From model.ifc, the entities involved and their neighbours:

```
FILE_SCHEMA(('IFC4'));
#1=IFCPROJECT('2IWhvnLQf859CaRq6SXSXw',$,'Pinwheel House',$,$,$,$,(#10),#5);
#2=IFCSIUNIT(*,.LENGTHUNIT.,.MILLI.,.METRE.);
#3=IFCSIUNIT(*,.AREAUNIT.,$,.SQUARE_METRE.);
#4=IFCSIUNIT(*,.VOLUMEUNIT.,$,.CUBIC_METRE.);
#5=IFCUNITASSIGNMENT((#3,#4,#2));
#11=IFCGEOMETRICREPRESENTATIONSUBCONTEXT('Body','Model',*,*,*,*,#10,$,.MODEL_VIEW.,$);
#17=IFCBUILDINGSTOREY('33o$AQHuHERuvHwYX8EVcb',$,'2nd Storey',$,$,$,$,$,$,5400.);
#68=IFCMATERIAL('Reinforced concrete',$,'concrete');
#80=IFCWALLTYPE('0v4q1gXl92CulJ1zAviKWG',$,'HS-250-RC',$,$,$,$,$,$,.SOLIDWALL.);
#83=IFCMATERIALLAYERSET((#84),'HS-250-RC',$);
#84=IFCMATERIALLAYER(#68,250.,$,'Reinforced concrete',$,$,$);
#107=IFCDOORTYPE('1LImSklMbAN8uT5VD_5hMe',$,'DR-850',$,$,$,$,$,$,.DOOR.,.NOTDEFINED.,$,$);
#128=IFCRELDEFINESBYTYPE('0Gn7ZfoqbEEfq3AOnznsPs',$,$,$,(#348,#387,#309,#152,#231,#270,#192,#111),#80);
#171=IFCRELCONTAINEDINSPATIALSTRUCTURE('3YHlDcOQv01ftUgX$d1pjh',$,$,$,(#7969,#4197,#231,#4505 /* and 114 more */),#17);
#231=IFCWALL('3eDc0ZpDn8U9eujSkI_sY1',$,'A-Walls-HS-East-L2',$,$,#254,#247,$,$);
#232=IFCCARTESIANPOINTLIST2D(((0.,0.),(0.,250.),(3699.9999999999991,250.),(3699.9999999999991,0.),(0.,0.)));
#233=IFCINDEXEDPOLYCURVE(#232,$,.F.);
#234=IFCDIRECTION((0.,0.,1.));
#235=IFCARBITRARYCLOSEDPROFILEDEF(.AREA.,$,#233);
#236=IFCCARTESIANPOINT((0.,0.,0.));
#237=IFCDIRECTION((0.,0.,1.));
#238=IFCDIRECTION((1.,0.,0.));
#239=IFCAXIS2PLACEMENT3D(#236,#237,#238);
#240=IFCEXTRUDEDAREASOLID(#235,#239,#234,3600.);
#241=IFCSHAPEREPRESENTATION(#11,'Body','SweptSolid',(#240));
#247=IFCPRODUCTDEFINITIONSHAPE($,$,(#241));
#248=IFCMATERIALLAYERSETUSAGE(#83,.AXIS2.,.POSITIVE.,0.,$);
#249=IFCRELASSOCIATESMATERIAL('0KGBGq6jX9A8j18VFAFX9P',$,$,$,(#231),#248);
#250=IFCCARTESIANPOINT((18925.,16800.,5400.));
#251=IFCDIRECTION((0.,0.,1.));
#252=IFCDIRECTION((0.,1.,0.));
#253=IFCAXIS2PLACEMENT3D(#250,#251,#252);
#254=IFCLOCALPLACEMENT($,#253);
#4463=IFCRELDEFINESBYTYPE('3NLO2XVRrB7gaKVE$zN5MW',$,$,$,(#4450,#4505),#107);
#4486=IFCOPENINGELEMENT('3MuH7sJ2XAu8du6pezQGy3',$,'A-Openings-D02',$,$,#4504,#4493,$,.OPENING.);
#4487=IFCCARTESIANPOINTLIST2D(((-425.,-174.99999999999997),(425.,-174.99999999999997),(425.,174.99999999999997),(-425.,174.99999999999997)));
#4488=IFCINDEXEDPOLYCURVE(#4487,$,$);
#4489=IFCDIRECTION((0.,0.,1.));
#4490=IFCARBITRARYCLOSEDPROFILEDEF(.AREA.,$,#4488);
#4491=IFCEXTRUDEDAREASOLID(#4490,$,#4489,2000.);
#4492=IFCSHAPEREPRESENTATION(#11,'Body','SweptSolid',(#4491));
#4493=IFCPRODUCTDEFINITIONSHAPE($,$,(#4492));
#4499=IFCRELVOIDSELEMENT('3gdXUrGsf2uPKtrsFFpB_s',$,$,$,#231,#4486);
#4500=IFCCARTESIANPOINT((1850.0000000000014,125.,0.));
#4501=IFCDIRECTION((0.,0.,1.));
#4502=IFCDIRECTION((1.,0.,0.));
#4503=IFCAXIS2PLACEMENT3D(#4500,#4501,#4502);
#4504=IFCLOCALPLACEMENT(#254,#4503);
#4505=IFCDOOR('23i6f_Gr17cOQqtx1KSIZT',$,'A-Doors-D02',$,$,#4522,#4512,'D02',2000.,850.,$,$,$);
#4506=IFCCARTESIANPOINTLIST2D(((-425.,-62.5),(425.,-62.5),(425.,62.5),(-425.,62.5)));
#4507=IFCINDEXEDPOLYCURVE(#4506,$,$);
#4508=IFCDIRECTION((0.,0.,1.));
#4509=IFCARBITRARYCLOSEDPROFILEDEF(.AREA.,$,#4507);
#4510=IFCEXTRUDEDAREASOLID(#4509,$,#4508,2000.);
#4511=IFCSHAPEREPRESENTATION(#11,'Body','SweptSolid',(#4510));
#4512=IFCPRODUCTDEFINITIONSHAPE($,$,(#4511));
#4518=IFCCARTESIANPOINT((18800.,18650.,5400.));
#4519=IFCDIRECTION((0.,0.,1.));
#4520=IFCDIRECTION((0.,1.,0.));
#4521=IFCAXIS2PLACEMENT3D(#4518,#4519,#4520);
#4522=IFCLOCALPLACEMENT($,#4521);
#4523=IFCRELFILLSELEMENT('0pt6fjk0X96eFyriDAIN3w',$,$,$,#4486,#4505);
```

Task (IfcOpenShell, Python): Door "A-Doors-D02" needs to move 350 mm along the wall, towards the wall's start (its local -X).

```python
import ifcopenshell
import ifcopenshell.api.geometry
import ifcopenshell.util.placement
import ifcopenshell.util.unit

model = ifcopenshell.open("model.ifc")
unit_scale = ifcopenshell.util.unit.calculate_unit_scale(model)

door = model.by_guid("23i6f_Gr17cOQqtx1KSIZT")
opening = door.FillsVoids[0].RelatingOpeningElement
wall = opening.VoidsElements[0].RelatingBuildingElement

wall_matrix = ifcopenshell.util.placement.get_local_placement(wall.ObjectPlacement)
shift = wall_matrix[:3, 0] * -0.35 / unit_scale
before = ifcopenshell.util.placement.get_local_placement(door.ObjectPlacement)[:3, 3].copy()

# The door is not placed relative to its opening, so move both.
for product in (opening, door):
    matrix = ifcopenshell.util.placement.get_local_placement(product.ObjectPlacement)
    matrix[:3, 3] += shift
    ifcopenshell.api.geometry.edit_object_placement(model, product=product, matrix=matrix, is_si=False)

after = ifcopenshell.util.placement.get_local_placement(door.ObjectPlacement)[:3, 3]
print("door moved by", (after - before).round(3) + 0.0)

model.write("model-out.ifc")
```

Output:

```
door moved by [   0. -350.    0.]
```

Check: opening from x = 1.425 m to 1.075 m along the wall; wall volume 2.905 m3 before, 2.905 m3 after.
